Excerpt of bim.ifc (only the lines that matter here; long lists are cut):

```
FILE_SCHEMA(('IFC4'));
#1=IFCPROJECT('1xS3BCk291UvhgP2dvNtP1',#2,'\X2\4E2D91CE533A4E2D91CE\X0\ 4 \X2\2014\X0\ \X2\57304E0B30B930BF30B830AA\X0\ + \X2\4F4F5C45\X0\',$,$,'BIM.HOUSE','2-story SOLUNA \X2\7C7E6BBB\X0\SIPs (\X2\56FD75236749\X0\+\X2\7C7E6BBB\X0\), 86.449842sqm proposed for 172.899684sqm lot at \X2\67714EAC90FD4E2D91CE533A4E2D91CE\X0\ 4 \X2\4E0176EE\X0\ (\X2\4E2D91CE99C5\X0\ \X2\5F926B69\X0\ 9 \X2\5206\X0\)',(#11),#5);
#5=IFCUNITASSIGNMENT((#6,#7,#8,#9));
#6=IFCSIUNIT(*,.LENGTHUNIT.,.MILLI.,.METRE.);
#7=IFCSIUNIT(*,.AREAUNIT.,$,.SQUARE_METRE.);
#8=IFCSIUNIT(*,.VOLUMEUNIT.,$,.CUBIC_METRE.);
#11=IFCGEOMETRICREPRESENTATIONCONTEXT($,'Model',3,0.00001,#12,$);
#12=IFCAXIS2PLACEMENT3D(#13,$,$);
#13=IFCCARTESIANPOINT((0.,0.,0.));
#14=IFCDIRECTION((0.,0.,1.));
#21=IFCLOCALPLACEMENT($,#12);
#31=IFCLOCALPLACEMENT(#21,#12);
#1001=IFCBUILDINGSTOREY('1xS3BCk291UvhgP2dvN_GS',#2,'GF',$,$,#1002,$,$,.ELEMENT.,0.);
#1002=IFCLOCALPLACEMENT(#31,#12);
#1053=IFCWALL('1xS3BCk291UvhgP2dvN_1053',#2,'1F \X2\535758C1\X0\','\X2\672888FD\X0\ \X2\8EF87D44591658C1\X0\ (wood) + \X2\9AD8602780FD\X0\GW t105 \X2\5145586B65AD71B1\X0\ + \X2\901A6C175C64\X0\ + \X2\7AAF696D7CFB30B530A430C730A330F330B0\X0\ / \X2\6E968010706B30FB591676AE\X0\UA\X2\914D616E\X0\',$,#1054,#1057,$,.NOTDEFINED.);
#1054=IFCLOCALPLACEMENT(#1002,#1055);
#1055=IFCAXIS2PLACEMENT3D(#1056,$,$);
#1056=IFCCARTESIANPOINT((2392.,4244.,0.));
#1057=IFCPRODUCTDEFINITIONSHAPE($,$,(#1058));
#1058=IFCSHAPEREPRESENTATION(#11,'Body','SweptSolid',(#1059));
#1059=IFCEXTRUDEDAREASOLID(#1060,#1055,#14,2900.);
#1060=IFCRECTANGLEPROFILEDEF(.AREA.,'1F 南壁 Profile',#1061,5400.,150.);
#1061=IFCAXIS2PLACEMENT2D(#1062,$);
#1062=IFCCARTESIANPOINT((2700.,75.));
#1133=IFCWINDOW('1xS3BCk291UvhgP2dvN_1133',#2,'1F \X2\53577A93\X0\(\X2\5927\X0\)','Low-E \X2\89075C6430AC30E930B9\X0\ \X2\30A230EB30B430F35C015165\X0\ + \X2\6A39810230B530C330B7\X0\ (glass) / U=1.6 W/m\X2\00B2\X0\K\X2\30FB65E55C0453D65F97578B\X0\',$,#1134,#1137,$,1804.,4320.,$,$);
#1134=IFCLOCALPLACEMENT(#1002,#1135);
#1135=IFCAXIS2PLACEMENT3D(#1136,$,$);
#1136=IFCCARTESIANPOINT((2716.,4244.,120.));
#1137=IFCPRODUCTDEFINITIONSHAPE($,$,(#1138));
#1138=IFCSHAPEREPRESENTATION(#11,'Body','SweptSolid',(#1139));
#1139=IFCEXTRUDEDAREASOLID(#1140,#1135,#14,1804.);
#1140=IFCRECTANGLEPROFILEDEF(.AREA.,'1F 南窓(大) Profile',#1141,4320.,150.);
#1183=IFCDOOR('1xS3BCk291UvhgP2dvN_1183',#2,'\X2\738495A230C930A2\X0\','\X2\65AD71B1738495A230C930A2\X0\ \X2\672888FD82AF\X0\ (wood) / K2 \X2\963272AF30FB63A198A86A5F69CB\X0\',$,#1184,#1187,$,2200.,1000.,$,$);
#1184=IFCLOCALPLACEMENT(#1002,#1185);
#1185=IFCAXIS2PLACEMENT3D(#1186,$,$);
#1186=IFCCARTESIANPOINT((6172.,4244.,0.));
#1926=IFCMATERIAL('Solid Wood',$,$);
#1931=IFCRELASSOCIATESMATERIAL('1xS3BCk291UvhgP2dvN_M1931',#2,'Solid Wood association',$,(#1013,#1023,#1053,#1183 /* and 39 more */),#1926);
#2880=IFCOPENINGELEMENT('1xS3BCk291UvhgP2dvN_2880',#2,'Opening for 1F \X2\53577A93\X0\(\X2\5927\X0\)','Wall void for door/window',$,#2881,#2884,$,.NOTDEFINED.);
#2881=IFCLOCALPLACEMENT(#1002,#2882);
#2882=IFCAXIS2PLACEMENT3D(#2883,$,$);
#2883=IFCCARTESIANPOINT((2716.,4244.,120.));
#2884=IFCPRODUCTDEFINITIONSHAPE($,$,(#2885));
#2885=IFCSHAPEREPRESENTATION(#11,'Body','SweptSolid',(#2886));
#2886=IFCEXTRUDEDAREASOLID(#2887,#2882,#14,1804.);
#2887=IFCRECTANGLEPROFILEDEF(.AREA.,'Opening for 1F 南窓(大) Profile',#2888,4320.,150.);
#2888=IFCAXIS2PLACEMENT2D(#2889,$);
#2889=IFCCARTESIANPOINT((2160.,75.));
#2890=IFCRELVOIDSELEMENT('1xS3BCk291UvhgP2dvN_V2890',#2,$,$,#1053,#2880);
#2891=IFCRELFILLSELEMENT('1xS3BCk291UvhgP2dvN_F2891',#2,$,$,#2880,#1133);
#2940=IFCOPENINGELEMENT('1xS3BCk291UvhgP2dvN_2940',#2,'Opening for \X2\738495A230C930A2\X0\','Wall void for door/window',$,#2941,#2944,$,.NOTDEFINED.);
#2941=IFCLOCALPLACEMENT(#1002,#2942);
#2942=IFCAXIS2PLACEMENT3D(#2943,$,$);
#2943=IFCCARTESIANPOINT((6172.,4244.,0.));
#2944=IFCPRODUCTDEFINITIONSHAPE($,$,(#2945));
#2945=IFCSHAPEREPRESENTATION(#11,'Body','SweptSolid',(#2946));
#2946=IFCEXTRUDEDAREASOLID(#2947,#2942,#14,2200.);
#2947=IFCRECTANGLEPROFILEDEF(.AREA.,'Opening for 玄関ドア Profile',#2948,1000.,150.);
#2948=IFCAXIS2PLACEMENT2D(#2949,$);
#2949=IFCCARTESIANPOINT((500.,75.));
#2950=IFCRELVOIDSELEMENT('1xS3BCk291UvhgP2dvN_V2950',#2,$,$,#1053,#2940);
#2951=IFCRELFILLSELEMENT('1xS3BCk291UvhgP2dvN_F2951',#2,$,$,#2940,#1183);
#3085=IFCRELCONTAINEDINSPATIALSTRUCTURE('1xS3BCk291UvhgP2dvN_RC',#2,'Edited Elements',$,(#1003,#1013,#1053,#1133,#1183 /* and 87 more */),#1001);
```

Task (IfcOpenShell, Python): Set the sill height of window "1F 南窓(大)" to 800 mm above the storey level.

```python
import numpy as np
import ifcopenshell
import ifcopenshell.api.geometry
import ifcopenshell.geom
import ifcopenshell.util.element
import ifcopenshell.util.placement
import ifcopenshell.util.shape
import ifcopenshell.util.unit

model = ifcopenshell.open("bim.ifc")
unit_scale = ifcopenshell.util.unit.calculate_unit_scale(model)

window = model.by_guid("1xS3BCk291UvhgP2dvN_1133")
opening = window.FillsVoids[0].RelatingOpeningElement
storey = ifcopenshell.util.element.get_container(window, ifc_class="IfcBuildingStorey")
level = ifcopenshell.util.placement.get_local_placement(storey.ObjectPlacement)[2, 3]

# The opening's origin need not be at the sill, so measure its lowest point.
shape = ifcopenshell.geom.create_shape(ifcopenshell.geom.settings(), opening)
bottom = ifcopenshell.util.shape.get_shape_bottom_elevation(shape, shape.geometry) / unit_scale
dz = level + 800.0 - bottom

shift = np.array([0.0, 0.0, dz])
# The window is not placed relative to its opening, so move both.
for product in (opening, window):
    matrix = ifcopenshell.util.placement.get_local_placement(product.ObjectPlacement)
    matrix[:3, 3] += shift
    ifcopenshell.api.geometry.edit_object_placement(model, product=product, matrix=matrix, is_si=False)

print(f"moved by {dz * unit_scale:+.3f} m")

model.write("bim_v2.ifc")
```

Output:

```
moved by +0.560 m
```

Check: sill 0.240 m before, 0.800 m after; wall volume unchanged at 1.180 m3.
